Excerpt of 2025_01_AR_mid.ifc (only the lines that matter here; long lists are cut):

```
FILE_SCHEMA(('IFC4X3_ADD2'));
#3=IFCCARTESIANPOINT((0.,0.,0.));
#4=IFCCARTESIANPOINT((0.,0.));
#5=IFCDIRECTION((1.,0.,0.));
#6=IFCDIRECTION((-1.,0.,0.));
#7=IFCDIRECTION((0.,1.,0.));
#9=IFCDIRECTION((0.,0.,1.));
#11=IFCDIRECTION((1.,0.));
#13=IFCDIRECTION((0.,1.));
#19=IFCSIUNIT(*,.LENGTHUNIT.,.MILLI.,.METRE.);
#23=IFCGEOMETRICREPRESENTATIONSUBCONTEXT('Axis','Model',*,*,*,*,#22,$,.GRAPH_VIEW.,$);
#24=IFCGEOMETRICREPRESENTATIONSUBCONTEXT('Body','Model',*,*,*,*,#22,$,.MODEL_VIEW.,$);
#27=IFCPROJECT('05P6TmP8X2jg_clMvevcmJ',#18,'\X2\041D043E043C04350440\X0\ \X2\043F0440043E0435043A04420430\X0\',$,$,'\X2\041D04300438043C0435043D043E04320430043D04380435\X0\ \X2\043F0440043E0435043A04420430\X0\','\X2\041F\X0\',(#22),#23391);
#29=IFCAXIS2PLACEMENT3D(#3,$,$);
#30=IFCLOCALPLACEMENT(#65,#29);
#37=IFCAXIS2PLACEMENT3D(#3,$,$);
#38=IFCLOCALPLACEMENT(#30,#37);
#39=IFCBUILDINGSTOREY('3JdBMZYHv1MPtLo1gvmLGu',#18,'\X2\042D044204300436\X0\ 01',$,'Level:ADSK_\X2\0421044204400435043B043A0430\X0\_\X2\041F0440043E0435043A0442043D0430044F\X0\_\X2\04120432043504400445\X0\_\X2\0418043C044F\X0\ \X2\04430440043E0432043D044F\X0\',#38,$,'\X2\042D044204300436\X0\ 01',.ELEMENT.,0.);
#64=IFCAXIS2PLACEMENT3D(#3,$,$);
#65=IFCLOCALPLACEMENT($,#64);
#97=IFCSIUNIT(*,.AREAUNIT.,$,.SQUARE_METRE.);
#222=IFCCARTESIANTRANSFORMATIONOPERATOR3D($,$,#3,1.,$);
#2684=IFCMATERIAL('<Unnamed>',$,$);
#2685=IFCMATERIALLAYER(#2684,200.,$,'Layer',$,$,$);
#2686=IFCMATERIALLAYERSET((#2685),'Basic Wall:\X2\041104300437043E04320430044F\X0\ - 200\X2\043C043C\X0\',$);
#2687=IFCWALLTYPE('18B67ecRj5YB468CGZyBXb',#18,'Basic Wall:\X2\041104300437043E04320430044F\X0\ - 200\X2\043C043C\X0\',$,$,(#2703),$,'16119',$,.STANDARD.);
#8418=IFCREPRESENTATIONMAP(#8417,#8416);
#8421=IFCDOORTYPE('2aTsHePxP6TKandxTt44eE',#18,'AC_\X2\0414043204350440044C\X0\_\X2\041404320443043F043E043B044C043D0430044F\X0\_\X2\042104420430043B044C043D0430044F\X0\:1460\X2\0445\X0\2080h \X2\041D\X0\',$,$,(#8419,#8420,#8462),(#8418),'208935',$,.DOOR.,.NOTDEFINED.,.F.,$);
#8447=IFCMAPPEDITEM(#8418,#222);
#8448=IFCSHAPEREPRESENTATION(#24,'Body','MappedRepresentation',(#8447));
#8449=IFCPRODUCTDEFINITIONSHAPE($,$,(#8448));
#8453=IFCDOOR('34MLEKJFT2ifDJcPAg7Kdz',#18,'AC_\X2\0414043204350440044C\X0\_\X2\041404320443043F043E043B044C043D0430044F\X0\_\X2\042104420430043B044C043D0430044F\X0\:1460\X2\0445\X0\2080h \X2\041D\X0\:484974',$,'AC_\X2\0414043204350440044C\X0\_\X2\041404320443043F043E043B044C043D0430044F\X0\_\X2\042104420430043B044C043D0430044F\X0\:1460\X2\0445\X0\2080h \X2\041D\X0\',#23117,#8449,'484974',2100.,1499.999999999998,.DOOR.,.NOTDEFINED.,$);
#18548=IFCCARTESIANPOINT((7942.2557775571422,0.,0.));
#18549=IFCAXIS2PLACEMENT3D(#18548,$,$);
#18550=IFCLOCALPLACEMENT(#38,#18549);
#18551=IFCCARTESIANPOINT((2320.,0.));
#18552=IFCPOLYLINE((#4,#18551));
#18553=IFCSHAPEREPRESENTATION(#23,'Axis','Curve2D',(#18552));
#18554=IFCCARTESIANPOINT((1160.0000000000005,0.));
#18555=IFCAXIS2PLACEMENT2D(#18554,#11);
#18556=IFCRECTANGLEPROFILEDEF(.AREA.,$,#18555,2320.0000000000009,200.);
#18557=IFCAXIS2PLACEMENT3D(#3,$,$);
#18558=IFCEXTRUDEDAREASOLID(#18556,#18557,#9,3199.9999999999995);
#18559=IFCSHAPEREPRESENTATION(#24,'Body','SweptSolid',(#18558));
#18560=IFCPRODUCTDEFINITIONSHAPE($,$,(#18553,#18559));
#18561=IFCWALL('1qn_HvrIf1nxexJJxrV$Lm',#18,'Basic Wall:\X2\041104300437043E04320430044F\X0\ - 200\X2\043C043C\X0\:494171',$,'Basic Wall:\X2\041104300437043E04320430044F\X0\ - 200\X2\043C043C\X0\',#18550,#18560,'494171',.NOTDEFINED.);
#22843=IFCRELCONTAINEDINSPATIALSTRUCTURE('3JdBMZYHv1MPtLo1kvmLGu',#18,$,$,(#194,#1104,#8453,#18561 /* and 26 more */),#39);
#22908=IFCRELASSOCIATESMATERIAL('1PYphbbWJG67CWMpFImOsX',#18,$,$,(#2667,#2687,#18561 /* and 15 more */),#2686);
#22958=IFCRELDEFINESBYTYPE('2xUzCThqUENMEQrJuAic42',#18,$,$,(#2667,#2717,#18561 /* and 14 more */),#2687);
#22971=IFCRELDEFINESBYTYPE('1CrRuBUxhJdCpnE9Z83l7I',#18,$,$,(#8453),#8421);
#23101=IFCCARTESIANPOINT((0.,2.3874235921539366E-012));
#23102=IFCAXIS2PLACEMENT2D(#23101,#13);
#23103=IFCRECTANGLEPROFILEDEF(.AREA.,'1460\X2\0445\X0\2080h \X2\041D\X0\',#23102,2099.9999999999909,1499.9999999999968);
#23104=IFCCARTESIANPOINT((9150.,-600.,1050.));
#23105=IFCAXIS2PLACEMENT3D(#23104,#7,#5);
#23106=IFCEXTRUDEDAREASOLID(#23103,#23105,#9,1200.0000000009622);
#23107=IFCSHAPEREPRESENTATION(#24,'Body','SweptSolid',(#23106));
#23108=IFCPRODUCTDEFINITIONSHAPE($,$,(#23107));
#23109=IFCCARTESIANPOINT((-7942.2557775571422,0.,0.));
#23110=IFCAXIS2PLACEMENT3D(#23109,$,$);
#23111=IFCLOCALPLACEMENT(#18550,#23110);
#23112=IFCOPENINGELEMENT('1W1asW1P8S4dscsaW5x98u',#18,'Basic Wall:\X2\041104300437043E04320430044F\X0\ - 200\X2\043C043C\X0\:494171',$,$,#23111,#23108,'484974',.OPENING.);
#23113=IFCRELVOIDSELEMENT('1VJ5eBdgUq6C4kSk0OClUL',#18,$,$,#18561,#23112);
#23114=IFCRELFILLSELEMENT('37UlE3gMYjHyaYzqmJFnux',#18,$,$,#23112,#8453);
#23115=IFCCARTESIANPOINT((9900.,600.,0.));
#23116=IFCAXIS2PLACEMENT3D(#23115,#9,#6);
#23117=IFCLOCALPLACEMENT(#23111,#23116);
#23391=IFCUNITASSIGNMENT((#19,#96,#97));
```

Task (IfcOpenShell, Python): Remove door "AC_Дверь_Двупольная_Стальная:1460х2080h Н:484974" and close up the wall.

```python
import ifcopenshell
import ifcopenshell.api.feature
import ifcopenshell.api.root
import ifcopenshell.geom
import ifcopenshell.util.shape

model = ifcopenshell.open("2025_01_AR_mid.ifc")
settings = ifcopenshell.geom.settings()


def volume(element):
    """Net volume in cubic metres, openings subtracted."""
    shape = ifcopenshell.geom.create_shape(settings, element)
    return ifcopenshell.util.shape.get_volume(shape.geometry)


door = model.by_id(8453)
opening = door.FillsVoids[0].RelatingOpeningElement
wall = opening.VoidsElements[0].RelatingBuildingElement
before = volume(wall)

ifcopenshell.api.root.remove_product(model, product=door)
ifcopenshell.api.feature.remove_feature(model, feature=opening)

after = volume(wall)

print(f"wall volume {before:.3f} -> {after:.3f} m3")

model.write("2025_01_AR_mid_v2.ifc")
```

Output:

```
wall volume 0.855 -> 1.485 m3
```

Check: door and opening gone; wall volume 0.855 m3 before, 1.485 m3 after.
